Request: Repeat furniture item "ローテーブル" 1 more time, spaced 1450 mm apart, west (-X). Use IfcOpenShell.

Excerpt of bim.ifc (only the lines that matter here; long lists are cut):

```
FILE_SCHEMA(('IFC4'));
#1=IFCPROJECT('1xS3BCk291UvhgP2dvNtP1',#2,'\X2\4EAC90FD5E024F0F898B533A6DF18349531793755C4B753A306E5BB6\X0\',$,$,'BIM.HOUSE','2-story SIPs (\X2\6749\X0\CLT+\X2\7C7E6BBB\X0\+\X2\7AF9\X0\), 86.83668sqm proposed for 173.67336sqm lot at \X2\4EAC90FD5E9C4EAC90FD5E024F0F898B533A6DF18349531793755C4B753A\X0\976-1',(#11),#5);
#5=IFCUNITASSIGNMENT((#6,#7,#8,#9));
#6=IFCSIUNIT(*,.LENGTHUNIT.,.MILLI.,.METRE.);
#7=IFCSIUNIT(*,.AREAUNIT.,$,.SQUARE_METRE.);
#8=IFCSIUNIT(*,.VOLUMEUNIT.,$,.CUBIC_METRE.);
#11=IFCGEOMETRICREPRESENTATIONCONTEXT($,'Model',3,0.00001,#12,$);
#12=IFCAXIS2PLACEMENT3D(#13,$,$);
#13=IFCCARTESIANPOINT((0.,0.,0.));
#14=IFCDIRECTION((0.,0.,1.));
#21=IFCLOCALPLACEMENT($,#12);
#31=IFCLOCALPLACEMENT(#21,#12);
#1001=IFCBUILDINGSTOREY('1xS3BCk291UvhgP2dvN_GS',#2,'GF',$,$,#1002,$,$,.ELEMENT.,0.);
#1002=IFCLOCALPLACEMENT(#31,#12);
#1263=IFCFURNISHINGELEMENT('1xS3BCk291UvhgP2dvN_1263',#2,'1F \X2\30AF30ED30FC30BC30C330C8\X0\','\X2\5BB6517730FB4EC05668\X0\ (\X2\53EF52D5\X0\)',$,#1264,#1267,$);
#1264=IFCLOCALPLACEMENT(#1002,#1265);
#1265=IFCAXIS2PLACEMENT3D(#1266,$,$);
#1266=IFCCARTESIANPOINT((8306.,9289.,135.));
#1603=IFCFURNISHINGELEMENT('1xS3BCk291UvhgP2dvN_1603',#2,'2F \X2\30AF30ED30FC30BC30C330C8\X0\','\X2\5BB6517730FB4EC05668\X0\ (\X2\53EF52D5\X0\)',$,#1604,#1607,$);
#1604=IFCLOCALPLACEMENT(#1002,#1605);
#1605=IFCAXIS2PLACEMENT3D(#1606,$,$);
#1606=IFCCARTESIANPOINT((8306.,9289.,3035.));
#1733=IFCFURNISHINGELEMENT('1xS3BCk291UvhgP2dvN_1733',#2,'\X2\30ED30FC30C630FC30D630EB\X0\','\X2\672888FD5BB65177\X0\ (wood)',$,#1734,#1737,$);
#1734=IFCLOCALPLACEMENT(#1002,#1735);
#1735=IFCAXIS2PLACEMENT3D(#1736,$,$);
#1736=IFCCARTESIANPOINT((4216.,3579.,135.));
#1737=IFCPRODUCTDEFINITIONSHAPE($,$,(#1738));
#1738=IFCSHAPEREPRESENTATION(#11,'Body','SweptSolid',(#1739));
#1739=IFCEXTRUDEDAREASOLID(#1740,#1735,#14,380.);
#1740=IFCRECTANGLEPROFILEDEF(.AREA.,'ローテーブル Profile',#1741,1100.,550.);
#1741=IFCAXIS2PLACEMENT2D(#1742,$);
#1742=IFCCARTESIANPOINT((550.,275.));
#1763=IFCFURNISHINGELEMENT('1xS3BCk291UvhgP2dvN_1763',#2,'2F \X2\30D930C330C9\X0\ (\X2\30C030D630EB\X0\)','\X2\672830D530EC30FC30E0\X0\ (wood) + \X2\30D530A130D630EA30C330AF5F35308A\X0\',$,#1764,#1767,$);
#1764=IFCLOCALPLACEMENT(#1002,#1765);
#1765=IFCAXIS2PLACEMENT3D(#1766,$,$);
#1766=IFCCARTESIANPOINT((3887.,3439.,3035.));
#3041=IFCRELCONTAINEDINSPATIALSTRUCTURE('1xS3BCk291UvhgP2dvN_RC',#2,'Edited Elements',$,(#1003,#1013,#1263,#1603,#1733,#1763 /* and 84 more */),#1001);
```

```python
import numpy as np
import ifcopenshell
import ifcopenshell.api.geometry
import ifcopenshell.api.root
import ifcopenshell.util.element
import ifcopenshell.util.placement
import ifcopenshell.util.unit

model = ifcopenshell.open("bim.ifc")
unit_scale = ifcopenshell.util.unit.calculate_unit_scale(model)


def reuse_history(source, copy):
    """copy_class also copies each property set's owner history, people and application; keep the originals."""
    for rel in copy.IsDefinedBy:
        if rel.is_a("IfcRelDefinesByProperties") and (history := rel.RelatingPropertyDefinition.OwnerHistory):
            rel.RelatingPropertyDefinition.OwnerHistory = source.OwnerHistory
            ifcopenshell.util.element.remove_deep2(model, history)


source = model.by_guid("1xS3BCk291UvhgP2dvN_1733")
base = ifcopenshell.util.placement.get_local_placement(source.ObjectPlacement)
step = np.array([-1.0, 0.0, 0.0]) * 1.45 / unit_scale

for i in range(1, 2):
    copy = ifcopenshell.api.root.copy_class(model, product=source)
    copy.Representation = ifcopenshell.util.element.copy_deep(
        model, source.Representation, exclude=["IfcGeometricRepresentationContext", "IfcRepresentationMap"]
    )
    reuse_history(source, copy)
    matrix = base.copy()
    matrix[:3, 3] += i * step
    print("added at", matrix[:3, 3].round(3) + 0.0)
    ifcopenshell.api.geometry.edit_object_placement(model, product=copy, matrix=matrix, is_si=False)

model.write("bim_updated.ifc")
```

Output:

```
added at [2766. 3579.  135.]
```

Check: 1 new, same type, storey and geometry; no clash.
